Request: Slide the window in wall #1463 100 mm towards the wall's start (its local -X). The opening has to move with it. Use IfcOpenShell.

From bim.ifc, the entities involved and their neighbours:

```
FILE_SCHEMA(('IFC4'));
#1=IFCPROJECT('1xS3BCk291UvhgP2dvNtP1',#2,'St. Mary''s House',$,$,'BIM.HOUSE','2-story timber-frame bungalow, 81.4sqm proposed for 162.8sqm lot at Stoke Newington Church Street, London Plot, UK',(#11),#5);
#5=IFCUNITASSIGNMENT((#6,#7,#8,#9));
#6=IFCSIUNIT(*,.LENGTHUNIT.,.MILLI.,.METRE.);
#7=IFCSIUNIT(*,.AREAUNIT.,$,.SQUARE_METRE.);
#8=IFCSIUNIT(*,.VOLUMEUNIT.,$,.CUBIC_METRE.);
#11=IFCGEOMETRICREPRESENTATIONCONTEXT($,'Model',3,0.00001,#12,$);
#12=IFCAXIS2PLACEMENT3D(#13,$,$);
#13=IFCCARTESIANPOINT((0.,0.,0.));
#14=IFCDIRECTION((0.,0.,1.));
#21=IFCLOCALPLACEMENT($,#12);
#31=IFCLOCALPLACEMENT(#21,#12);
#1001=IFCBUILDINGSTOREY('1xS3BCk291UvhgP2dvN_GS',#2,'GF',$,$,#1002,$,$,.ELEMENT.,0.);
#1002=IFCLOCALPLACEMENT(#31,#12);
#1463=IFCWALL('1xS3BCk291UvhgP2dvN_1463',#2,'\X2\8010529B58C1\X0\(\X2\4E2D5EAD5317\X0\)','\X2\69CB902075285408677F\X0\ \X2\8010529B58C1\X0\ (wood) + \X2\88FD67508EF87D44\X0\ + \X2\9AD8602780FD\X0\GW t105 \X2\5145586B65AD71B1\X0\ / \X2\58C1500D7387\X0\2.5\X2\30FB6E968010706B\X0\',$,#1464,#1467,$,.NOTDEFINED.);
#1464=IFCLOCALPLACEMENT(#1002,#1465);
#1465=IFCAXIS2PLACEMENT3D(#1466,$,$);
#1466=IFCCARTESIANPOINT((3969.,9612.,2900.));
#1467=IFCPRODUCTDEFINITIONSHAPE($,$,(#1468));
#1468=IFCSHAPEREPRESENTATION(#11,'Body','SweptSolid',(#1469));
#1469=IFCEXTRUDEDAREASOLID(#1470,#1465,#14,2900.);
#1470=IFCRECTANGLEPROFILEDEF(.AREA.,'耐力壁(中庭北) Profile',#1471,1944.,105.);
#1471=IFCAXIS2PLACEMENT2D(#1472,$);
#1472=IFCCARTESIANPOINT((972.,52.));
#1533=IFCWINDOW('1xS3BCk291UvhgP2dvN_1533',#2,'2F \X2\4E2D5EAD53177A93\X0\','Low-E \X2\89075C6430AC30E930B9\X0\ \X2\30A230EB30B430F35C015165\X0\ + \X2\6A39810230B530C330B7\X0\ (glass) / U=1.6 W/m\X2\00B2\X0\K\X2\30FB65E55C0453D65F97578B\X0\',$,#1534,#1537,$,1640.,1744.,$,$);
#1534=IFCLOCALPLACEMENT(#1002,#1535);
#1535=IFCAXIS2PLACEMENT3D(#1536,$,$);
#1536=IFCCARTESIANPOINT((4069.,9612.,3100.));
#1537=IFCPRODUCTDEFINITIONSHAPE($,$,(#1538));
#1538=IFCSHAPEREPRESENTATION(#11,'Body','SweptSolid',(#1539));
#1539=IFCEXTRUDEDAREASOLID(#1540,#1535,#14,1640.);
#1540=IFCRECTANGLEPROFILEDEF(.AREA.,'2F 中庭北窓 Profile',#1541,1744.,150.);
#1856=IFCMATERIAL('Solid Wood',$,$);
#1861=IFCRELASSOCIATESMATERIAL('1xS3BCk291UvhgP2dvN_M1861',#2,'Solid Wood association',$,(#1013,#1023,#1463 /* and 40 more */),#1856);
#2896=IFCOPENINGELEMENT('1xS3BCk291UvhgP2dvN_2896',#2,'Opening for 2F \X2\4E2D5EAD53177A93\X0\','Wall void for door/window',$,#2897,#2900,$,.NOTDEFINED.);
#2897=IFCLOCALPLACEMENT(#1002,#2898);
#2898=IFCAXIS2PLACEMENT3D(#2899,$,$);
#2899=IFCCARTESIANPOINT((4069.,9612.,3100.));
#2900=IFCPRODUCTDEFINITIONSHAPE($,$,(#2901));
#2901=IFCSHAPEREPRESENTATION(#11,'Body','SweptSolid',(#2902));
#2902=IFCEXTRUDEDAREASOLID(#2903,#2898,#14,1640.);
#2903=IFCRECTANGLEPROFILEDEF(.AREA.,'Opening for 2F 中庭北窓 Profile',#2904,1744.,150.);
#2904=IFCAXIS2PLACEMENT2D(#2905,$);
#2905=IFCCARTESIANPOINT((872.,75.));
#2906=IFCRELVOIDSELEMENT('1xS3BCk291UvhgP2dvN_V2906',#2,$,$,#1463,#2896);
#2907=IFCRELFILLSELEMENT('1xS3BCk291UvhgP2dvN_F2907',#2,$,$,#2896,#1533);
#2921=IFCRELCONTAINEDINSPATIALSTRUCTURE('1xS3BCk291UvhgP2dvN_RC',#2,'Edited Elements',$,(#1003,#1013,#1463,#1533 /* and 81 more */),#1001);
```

```python
import ifcopenshell
import ifcopenshell.api.geometry
import ifcopenshell.util.placement
import ifcopenshell.util.unit

model = ifcopenshell.open("bim.ifc")
unit_scale = ifcopenshell.util.unit.calculate_unit_scale(model)

window = model.by_guid("1xS3BCk291UvhgP2dvN_1533")
opening = window.FillsVoids[0].RelatingOpeningElement
wall = opening.VoidsElements[0].RelatingBuildingElement

wall_matrix = ifcopenshell.util.placement.get_local_placement(wall.ObjectPlacement)
shift = wall_matrix[:3, 0] * -0.1 / unit_scale
before = ifcopenshell.util.placement.get_local_placement(window.ObjectPlacement)[:3, 3].copy()

# The window is not placed relative to its opening, so move both.
for product in (opening, window):
    matrix = ifcopenshell.util.placement.get_local_placement(product.ObjectPlacement)
    matrix[:3, 3] += shift
    ifcopenshell.api.geometry.edit_object_placement(model, product=product, matrix=matrix, is_si=False)

after = ifcopenshell.util.placement.get_local_placement(window.ObjectPlacement)[:3, 3]
print("window moved by", (after - before).round(3) + 0.0)

model.write("bim_v2.ifc")
```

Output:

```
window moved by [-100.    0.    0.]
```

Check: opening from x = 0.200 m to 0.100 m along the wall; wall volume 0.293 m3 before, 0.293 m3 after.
